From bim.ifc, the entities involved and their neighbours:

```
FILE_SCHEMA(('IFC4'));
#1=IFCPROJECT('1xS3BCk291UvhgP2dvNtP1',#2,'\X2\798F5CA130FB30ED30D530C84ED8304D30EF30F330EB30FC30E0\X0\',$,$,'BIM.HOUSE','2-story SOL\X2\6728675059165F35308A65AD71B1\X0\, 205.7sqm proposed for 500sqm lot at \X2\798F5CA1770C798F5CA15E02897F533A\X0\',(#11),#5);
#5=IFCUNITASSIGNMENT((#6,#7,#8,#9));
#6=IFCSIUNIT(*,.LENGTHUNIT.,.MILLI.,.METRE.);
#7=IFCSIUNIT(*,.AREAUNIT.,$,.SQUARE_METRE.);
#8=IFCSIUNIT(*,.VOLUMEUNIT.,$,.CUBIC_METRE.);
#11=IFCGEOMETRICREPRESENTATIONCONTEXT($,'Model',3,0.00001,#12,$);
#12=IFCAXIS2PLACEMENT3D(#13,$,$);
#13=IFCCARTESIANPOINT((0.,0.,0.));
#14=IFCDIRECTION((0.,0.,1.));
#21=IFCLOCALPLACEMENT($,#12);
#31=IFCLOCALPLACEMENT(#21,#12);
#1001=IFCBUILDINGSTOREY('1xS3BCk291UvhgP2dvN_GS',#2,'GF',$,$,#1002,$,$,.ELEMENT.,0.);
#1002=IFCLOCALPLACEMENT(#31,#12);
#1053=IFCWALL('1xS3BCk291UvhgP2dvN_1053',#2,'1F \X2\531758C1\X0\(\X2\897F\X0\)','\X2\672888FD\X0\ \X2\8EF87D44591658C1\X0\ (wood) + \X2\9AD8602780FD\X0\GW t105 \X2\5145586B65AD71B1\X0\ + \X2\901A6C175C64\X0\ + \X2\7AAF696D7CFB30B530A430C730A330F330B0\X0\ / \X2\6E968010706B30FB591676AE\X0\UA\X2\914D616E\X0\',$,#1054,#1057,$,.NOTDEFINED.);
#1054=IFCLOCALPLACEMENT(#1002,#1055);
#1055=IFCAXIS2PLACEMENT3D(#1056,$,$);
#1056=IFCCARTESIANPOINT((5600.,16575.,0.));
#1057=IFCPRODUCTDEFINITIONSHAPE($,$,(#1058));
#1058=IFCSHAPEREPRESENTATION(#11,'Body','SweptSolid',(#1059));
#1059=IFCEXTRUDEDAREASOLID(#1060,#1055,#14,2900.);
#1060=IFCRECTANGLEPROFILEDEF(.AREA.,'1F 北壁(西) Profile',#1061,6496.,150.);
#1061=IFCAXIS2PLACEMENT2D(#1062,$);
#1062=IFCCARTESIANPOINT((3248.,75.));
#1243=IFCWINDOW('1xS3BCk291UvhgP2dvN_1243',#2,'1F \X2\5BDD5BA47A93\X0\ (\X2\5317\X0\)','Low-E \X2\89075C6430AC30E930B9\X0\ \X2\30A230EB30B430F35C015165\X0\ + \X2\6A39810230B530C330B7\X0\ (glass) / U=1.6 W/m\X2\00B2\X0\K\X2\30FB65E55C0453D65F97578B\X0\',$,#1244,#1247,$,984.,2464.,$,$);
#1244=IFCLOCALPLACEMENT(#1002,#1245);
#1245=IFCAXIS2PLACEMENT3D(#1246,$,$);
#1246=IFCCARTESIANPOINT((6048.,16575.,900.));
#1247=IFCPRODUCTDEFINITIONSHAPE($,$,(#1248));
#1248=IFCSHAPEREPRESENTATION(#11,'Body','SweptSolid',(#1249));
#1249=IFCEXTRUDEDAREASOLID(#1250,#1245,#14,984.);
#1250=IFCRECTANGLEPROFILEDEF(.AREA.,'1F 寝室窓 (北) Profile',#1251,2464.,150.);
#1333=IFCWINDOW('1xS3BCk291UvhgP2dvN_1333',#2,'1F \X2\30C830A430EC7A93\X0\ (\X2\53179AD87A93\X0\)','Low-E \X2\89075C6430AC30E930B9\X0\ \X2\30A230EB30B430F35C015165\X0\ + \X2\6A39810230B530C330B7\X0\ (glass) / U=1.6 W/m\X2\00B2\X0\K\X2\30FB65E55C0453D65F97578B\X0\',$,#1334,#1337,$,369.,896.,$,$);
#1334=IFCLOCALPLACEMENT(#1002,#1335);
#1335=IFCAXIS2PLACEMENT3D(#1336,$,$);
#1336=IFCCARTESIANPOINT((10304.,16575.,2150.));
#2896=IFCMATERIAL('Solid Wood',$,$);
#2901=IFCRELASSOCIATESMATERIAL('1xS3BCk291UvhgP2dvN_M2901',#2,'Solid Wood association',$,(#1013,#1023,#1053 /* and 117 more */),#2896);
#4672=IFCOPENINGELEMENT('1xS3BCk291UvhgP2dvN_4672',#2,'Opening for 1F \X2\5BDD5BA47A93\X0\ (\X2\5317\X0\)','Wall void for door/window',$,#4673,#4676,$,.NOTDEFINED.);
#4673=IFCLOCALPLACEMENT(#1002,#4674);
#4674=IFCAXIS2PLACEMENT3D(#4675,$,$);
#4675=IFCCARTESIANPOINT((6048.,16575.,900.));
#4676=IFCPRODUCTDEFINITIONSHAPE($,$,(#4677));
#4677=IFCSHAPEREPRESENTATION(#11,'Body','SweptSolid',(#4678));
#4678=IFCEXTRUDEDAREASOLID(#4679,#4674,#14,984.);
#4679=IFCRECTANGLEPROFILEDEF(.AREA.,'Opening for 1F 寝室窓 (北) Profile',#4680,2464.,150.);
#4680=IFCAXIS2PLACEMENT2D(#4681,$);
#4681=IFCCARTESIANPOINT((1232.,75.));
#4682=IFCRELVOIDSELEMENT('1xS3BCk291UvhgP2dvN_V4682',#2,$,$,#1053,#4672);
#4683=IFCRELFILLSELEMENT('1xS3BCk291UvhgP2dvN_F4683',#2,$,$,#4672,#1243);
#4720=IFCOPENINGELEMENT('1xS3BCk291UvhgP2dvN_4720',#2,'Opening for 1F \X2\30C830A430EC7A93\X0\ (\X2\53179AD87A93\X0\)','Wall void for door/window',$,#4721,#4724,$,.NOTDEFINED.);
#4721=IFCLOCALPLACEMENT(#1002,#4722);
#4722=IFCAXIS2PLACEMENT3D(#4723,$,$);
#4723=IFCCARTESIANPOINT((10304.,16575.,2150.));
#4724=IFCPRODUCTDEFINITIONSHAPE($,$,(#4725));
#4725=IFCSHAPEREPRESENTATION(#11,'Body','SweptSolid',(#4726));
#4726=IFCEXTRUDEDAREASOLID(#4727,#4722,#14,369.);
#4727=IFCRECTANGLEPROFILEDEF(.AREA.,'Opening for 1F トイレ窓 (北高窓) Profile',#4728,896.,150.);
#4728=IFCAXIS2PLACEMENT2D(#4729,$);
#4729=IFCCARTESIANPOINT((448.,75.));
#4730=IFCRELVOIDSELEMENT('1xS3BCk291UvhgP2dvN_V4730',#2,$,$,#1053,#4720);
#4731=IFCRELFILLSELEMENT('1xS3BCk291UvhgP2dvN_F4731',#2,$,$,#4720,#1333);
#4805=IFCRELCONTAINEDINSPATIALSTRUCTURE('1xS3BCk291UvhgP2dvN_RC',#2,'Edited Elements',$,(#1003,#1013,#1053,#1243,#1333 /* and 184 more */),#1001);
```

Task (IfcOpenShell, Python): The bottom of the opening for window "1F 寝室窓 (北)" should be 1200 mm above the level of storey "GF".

```python
import numpy as np
import ifcopenshell
import ifcopenshell.api.geometry
import ifcopenshell.geom
import ifcopenshell.util.element
import ifcopenshell.util.placement
import ifcopenshell.util.shape
import ifcopenshell.util.unit

model = ifcopenshell.open("bim.ifc")
unit_scale = ifcopenshell.util.unit.calculate_unit_scale(model)

window = model.by_id(1243)
opening = window.FillsVoids[0].RelatingOpeningElement
storey = ifcopenshell.util.element.get_container(window, ifc_class="IfcBuildingStorey")
level = ifcopenshell.util.placement.get_local_placement(storey.ObjectPlacement)[2, 3]

# The opening's origin need not be at the sill, so measure its lowest point.
shape = ifcopenshell.geom.create_shape(ifcopenshell.geom.settings(), opening)
bottom = ifcopenshell.util.shape.get_shape_bottom_elevation(shape, shape.geometry) / unit_scale
dz = level + 1200.0 - bottom

shift = np.array([0.0, 0.0, dz])
# The window is not placed relative to its opening, so move both.
for product in (opening, window):
    matrix = ifcopenshell.util.placement.get_local_placement(product.ObjectPlacement)
    matrix[:3, 3] += shift
    ifcopenshell.api.geometry.edit_object_placement(model, product=product, matrix=matrix, is_si=False)

print(f"moved by {dz * unit_scale:+.3f} m")

model.write("bim_v2.ifc")
```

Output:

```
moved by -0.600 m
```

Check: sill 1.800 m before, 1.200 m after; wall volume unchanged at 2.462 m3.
